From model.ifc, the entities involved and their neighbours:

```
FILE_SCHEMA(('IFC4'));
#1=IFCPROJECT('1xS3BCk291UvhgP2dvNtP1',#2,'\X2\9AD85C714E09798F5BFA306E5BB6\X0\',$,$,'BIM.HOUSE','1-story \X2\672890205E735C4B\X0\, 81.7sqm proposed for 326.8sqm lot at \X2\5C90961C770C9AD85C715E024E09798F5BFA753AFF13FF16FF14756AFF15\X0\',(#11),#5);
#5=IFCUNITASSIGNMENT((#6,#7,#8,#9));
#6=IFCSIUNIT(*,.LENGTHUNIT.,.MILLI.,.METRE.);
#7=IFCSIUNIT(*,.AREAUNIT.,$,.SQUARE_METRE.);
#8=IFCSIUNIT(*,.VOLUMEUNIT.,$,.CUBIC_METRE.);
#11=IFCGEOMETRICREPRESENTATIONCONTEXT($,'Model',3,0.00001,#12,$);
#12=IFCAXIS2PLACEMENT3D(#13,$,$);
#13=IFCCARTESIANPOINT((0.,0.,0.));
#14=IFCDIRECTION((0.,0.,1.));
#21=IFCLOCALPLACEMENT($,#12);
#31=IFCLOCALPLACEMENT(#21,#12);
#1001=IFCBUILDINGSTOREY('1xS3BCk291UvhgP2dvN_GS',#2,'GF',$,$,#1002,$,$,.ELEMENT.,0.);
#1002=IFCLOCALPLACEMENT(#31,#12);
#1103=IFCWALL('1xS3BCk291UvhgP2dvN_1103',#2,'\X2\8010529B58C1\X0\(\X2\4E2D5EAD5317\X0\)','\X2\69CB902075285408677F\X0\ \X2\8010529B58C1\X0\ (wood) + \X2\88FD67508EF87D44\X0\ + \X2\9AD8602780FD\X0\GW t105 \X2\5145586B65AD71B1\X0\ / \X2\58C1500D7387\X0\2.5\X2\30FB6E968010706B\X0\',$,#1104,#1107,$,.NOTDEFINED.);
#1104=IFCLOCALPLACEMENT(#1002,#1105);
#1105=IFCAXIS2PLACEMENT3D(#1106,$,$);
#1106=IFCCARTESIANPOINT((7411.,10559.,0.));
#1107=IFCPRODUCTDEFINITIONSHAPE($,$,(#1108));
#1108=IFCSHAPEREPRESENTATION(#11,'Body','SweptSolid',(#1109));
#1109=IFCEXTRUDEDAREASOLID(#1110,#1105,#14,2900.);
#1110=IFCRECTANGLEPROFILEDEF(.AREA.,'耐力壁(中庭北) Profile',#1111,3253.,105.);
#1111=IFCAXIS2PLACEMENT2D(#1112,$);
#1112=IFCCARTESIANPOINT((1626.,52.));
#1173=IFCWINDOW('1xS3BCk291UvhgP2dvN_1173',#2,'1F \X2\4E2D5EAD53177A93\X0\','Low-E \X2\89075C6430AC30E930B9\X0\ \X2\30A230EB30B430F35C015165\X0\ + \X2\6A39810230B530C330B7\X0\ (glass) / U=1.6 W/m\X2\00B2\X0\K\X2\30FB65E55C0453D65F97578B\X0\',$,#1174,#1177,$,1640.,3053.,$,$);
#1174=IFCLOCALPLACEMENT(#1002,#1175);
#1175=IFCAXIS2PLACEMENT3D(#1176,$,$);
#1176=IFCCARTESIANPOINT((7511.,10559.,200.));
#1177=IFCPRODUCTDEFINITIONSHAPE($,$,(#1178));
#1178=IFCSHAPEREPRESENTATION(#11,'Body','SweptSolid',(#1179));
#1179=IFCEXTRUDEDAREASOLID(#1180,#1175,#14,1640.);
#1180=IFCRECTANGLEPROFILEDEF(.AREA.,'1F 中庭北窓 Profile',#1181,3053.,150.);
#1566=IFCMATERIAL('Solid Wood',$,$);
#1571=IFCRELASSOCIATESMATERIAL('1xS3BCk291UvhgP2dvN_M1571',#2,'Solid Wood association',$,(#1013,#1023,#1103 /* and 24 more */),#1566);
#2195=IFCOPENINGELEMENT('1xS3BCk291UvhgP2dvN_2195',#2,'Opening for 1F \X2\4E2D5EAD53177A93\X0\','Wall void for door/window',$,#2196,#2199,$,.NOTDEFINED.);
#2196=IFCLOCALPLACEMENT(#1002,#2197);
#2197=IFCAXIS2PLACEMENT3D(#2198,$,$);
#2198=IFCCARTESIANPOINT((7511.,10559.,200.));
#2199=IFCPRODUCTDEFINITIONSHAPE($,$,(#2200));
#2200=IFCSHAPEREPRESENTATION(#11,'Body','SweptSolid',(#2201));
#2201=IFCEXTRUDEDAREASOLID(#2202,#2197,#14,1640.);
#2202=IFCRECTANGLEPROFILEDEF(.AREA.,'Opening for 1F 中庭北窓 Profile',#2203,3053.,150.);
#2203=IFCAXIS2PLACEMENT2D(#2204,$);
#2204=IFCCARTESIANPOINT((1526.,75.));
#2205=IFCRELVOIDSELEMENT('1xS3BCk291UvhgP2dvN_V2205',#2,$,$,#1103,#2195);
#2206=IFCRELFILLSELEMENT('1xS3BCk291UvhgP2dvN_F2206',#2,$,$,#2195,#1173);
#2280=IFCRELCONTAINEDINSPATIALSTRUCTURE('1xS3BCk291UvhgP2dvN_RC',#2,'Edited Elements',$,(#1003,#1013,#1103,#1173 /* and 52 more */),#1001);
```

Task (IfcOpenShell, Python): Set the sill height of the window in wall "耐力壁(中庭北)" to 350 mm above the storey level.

```python
import numpy as np
import ifcopenshell
import ifcopenshell.api.geometry
import ifcopenshell.geom
import ifcopenshell.util.element
import ifcopenshell.util.placement
import ifcopenshell.util.shape
import ifcopenshell.util.unit

model = ifcopenshell.open("model.ifc")
unit_scale = ifcopenshell.util.unit.calculate_unit_scale(model)

window = model.by_guid("1xS3BCk291UvhgP2dvN_1173")
opening = window.FillsVoids[0].RelatingOpeningElement
storey = ifcopenshell.util.element.get_container(window, ifc_class="IfcBuildingStorey")
level = ifcopenshell.util.placement.get_local_placement(storey.ObjectPlacement)[2, 3]

# The opening's origin need not be at the sill, so measure its lowest point.
shape = ifcopenshell.geom.create_shape(ifcopenshell.geom.settings(), opening)
bottom = ifcopenshell.util.shape.get_shape_bottom_elevation(shape, shape.geometry) / unit_scale
dz = level + 350.0 - bottom

shift = np.array([0.0, 0.0, dz])
# The window is not placed relative to its opening, so move both.
for product in (opening, window):
    matrix = ifcopenshell.util.placement.get_local_placement(product.ObjectPlacement)
    matrix[:3, 3] += shift
    ifcopenshell.api.geometry.edit_object_placement(model, product=product, matrix=matrix, is_si=False)

print(f"moved by {dz * unit_scale:+.3f} m")

model.write("model_updated.ifc")
```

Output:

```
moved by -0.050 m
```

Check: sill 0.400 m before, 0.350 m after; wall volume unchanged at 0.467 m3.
